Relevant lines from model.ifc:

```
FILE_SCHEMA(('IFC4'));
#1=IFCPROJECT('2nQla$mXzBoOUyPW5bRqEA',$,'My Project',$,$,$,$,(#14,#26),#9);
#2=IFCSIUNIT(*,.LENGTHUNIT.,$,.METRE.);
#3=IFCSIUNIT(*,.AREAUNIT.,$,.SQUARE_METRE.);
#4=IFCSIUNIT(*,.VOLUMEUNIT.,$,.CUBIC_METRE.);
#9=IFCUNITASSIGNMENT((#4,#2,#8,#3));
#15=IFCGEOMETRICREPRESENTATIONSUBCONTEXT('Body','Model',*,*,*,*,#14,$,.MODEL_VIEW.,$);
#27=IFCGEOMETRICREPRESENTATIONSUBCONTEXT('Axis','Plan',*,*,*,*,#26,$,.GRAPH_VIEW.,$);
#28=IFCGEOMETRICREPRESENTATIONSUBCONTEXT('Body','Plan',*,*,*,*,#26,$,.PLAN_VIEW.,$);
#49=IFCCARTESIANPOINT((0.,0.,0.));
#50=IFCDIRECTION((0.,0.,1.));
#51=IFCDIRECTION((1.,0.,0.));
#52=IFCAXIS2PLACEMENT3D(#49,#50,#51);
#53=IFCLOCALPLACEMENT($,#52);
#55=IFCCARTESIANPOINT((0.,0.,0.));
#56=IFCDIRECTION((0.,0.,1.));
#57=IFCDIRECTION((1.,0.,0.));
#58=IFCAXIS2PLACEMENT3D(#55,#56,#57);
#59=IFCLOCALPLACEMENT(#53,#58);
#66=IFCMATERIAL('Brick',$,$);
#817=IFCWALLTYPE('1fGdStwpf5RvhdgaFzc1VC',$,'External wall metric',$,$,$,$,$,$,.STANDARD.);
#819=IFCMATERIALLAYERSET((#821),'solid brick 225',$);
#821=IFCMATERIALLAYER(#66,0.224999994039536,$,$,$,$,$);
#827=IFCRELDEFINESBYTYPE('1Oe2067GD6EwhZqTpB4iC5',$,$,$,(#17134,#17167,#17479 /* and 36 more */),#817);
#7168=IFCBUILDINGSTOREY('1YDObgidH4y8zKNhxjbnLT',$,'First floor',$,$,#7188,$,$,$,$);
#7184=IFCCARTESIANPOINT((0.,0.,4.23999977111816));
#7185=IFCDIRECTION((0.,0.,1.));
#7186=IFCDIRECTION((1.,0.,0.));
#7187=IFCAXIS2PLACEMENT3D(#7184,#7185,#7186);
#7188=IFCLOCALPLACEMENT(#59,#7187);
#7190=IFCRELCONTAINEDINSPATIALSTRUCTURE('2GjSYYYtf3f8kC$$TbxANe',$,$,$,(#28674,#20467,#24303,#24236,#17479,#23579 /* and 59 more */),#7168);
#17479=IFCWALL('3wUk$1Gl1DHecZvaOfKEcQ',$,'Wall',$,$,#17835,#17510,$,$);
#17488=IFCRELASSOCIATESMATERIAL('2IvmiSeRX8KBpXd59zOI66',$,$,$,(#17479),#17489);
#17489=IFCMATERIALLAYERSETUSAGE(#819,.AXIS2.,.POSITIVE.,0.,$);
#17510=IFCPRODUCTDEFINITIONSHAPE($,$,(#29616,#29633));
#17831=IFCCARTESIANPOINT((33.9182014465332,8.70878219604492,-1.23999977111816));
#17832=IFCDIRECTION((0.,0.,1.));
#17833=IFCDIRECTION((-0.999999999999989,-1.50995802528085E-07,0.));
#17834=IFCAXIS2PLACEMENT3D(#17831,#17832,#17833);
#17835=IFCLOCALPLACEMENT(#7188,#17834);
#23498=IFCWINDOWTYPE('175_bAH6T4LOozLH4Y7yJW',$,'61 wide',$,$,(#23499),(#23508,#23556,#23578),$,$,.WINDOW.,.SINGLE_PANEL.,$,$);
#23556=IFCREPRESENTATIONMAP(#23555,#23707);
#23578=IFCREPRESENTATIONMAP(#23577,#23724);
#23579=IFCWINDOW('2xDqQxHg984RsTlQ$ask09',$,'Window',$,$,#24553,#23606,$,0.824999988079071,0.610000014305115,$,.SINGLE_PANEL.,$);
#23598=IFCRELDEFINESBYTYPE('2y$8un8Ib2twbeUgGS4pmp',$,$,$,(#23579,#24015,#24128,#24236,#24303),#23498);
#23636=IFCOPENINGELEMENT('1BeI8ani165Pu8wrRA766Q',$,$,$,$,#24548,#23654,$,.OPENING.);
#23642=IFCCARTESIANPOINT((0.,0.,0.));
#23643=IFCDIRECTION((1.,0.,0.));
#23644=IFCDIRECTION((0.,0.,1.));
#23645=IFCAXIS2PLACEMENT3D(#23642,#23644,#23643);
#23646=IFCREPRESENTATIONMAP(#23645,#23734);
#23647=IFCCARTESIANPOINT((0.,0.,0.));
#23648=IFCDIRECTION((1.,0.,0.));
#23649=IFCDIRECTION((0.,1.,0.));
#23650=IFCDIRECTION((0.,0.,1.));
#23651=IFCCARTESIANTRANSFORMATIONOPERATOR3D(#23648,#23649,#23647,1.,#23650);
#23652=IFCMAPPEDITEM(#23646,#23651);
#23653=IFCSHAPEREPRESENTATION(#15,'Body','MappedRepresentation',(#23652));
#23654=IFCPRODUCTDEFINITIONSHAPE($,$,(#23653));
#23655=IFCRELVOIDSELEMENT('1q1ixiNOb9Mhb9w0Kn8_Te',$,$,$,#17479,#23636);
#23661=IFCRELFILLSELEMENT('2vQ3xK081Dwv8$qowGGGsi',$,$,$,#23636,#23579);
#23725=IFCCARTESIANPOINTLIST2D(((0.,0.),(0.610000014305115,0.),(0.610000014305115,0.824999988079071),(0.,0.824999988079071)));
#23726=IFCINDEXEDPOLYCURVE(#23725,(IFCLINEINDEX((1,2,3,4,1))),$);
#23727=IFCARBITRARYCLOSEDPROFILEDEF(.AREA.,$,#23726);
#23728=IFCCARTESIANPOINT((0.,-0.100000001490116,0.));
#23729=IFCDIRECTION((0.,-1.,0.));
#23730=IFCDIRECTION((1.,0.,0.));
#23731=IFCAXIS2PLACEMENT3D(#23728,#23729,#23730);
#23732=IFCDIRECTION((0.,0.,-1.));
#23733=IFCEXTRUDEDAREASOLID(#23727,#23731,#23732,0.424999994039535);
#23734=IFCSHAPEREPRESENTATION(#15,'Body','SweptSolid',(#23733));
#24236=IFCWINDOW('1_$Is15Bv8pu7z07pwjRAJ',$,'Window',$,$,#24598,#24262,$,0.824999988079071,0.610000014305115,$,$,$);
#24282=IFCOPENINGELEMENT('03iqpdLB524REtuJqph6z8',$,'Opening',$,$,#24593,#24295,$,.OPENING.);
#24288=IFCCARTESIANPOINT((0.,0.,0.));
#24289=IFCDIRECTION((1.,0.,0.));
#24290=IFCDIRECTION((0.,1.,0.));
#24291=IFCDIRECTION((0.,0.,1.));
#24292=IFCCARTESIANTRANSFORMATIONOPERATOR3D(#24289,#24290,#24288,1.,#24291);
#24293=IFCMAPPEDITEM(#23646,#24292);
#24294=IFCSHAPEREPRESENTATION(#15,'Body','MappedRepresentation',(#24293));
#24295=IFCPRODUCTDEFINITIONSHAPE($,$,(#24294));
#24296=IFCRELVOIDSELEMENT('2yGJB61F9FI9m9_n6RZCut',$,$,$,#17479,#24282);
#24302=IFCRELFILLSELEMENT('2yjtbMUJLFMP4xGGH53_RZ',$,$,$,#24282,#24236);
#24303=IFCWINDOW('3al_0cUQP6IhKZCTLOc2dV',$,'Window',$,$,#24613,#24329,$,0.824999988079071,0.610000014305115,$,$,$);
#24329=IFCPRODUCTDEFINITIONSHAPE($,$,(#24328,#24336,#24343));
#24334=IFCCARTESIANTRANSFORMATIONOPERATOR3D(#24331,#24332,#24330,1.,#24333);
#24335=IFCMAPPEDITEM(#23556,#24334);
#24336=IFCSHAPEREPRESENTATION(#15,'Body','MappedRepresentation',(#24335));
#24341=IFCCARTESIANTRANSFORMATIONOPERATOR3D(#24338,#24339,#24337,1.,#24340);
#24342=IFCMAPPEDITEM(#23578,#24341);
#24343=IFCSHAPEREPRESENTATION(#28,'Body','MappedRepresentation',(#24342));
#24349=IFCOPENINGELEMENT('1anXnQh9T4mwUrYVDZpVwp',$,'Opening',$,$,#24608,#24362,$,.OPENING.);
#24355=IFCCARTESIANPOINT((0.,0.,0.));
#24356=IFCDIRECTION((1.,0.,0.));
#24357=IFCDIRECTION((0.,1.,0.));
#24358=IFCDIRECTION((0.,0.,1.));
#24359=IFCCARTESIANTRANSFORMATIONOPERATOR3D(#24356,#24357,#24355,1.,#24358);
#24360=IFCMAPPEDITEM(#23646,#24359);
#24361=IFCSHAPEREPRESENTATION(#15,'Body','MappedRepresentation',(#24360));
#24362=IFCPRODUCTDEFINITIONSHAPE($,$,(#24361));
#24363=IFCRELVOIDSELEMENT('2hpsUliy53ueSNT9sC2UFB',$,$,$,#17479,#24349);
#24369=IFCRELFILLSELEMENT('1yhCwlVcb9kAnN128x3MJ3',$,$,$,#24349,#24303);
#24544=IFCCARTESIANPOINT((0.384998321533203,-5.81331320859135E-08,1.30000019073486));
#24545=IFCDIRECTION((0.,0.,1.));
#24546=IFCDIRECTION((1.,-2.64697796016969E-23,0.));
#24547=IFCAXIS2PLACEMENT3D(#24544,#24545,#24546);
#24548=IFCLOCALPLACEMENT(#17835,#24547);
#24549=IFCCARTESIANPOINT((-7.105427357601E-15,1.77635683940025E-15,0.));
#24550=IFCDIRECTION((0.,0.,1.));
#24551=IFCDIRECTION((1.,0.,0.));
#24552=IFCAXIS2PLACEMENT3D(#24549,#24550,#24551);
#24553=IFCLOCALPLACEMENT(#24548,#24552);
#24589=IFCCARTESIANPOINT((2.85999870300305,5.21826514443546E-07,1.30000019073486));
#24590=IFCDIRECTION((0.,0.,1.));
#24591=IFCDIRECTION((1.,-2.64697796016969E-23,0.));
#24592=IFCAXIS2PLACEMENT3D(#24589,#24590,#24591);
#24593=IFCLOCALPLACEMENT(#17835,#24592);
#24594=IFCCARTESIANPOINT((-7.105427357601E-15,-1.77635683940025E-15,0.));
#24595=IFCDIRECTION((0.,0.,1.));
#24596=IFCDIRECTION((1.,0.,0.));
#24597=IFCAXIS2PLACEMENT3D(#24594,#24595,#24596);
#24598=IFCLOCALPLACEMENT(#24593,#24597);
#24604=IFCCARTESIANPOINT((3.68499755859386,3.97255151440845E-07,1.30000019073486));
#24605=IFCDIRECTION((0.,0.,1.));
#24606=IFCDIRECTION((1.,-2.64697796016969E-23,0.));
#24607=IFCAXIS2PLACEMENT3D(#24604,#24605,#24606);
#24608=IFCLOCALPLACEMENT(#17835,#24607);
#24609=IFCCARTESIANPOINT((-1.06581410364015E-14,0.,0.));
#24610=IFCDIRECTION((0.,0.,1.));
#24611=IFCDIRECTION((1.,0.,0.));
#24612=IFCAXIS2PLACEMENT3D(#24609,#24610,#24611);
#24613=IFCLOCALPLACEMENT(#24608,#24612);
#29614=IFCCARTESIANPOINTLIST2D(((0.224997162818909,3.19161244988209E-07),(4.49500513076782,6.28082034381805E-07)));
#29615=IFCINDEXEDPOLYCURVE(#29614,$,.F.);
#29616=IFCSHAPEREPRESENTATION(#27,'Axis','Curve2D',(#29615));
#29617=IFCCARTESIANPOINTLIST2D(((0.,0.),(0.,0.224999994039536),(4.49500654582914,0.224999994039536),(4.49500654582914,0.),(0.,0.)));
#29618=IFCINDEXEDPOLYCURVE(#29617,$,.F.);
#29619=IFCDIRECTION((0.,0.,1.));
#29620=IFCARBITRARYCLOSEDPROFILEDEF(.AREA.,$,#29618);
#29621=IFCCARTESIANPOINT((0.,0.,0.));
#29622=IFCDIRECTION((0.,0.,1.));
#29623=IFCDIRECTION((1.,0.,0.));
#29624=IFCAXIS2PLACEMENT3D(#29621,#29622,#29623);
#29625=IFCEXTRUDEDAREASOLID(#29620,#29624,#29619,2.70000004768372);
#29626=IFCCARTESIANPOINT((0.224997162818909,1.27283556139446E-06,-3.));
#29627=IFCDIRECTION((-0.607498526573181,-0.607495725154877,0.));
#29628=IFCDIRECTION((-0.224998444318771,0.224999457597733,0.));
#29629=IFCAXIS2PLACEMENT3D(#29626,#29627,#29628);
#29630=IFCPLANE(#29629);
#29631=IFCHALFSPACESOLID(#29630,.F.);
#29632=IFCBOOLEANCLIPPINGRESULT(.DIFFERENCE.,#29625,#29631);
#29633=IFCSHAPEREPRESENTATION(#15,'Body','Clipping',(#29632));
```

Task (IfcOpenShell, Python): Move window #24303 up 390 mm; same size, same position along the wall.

```python
import numpy as np
import ifcopenshell
import ifcopenshell.api.geometry
import ifcopenshell.util.placement
import ifcopenshell.util.unit

model = ifcopenshell.open("model.ifc")
unit_scale = ifcopenshell.util.unit.calculate_unit_scale(model)

window = model.by_guid("3al_0cUQP6IhKZCTLOc2dV")
opening = window.FillsVoids[0].RelatingOpeningElement
dz = 0.39

shift = np.array([0.0, 0.0, dz])
# The window is placed relative to its opening, so it follows when the opening moves.
matrix = ifcopenshell.util.placement.get_local_placement(opening.ObjectPlacement)
matrix[:3, 3] += shift
ifcopenshell.api.geometry.edit_object_placement(
    model, product=opening, matrix=matrix, is_si=False, should_transform_children=True
)

print(f"moved by {dz * unit_scale:+.3f} m")

model.write("model_edited.ifc")
```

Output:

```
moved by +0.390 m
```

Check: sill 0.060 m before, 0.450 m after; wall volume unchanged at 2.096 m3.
